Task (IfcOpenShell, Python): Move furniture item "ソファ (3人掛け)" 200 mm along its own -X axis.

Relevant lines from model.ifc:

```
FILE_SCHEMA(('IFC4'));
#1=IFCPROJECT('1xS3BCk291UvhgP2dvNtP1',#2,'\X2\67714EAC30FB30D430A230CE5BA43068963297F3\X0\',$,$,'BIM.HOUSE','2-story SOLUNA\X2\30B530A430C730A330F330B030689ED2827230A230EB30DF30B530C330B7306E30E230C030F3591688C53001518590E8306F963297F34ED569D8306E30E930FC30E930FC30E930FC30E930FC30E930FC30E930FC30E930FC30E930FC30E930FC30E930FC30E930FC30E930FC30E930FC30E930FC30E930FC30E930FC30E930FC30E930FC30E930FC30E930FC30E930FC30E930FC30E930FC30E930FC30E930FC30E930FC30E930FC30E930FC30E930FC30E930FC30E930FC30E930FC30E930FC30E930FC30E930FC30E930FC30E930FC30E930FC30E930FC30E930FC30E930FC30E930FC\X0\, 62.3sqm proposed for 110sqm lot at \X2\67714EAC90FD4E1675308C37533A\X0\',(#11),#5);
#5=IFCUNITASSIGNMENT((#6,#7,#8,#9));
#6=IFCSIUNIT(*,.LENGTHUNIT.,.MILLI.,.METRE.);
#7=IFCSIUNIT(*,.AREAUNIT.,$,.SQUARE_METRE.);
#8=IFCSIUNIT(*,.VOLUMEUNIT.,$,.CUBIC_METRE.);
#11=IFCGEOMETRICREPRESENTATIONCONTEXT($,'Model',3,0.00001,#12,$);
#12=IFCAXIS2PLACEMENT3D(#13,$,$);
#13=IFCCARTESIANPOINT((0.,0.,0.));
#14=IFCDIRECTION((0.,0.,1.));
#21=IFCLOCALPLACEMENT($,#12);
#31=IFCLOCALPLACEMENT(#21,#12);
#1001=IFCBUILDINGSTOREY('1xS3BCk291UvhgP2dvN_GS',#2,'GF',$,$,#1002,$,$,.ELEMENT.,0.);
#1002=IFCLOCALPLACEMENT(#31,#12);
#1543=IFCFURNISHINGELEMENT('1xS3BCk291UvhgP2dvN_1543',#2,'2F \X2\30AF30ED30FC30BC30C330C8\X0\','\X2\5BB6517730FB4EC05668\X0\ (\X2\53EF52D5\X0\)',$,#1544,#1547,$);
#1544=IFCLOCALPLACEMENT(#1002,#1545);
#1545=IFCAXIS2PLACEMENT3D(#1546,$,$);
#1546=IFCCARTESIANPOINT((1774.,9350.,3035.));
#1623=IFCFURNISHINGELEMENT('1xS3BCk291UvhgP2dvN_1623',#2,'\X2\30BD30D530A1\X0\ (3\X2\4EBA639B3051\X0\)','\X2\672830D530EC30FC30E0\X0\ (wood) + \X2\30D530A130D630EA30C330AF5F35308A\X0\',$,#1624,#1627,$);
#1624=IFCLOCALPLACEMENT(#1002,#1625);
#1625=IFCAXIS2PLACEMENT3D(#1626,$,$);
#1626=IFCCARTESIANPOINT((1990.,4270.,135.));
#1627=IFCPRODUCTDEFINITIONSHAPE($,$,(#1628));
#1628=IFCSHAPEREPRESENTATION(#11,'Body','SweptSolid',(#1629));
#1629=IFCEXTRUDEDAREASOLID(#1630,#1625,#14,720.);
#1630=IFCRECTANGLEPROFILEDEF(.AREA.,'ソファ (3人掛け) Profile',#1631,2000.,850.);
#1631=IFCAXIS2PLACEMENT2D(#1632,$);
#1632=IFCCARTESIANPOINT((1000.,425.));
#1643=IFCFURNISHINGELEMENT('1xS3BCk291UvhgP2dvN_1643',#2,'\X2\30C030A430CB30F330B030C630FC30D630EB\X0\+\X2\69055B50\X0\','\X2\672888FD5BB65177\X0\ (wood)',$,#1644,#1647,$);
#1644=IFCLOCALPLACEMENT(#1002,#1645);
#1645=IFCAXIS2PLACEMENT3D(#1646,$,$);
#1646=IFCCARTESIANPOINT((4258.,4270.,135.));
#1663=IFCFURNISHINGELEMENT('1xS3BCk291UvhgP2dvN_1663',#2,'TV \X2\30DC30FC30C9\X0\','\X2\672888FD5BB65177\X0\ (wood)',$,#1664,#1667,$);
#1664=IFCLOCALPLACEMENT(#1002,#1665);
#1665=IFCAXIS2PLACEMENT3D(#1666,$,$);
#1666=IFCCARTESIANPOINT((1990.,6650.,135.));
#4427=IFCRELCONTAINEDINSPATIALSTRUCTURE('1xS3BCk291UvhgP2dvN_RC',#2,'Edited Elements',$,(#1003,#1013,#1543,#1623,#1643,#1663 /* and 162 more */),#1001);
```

```python
import ifcopenshell
import ifcopenshell.api.geometry
import ifcopenshell.util.placement

model = ifcopenshell.open("model.ifc")

item = model.by_guid("1xS3BCk291UvhgP2dvN_1623")
matrix = ifcopenshell.util.placement.get_local_placement(item.ObjectPlacement)
matrix[:3, 3] -= matrix[:3, 0] * 200.0
ifcopenshell.api.geometry.edit_object_placement(model, product=item, matrix=matrix, is_si=False)

print(ifcopenshell.util.placement.get_local_placement(item.ObjectPlacement).round(3) + 0.0)

model.write("model-out.ifc")
```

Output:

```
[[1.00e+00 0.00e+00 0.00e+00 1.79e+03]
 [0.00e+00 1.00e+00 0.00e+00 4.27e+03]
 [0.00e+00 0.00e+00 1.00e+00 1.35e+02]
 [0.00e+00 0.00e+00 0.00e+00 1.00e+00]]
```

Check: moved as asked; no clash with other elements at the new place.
